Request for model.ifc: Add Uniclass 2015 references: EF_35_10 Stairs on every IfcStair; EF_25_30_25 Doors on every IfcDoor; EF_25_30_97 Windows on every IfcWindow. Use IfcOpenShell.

First a look at what the model holds.

```python
import ifcopenshell

model = ifcopenshell.open("model.ifc")
print(model.schema)
print("classifications:", [c.Name for c in model.by_type("IfcClassification")])
for ifc_class in ("IfcDoor", "IfcRoof", "IfcStair", "IfcWall", "IfcWindow"):
    print(ifc_class, len(model.by_type(ifc_class)))
```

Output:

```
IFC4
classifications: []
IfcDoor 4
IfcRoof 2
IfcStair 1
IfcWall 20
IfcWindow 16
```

```python
import ifcopenshell
import ifcopenshell.api.classification

model = ifcopenshell.open("model.ifc")

system = ifcopenshell.api.classification.add_classification(model, classification="Uniclass 2015")

codes = {
    "IfcStair": ("EF_35_10", "Stairs"),
    "IfcDoor": ("EF_25_30_25", "Doors"),
    "IfcWindow": ("EF_25_30_97", "Windows"),
}
for ifc_class, (code, name) in codes.items():
    products = model.by_type(ifc_class)
    ifcopenshell.api.classification.add_reference(
        model, products=products, classification=system, identification=code, name=name
    )
    print(code, len(products))

model.write("model_updated.ifc")
```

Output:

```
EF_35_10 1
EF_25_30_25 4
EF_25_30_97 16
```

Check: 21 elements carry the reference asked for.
